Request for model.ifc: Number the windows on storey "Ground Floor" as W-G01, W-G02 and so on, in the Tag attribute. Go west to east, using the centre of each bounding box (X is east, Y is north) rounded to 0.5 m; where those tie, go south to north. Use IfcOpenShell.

First a look at what the model holds.

```python
import ifcopenshell
import ifcopenshell.util.element
import ifcopenshell.util.placement

model = ifcopenshell.open("model.ifc")
print(model.schema)
storey = next(s for s in model.by_type("IfcBuildingStorey") if s.Name == "Ground Floor")
windows = [e for e in ifcopenshell.util.element.get_decomposition(storey) if e.is_a("IfcWindow")]
for e in sorted(windows, key=lambda e: e.id()):
    origin = ifcopenshell.util.placement.get_local_placement(e.ObjectPlacement)[:3, 3]
    print(e.id(), e.Tag, e.Name, origin.round(2) + 0.0, sep=" | ")
```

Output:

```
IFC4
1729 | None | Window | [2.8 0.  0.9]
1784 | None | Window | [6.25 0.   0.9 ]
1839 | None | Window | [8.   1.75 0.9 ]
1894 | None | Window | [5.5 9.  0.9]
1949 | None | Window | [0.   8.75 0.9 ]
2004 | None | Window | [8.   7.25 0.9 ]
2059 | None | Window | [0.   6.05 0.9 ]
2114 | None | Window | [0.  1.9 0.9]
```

```python
import ifcopenshell
import ifcopenshell.geom
import ifcopenshell.util.element
import ifcopenshell.util.shape

model = ifcopenshell.open("model.ifc")
settings = ifcopenshell.geom.settings()
settings.set("use-world-coords", True)


def centre(element):
    shape = ifcopenshell.geom.create_shape(settings, element)
    return ifcopenshell.util.shape.get_bbox_centroid(shape.geometry)


storey = next(s for s in model.by_type("IfcBuildingStorey") if s.Name == "Ground Floor")
windows = [e for e in ifcopenshell.util.element.get_decomposition(storey) if e.is_a("IfcWindow")]

# Insertion points can sit at a corner or the storey origin, so sort by the geometry (in metres).
centres = {e: centre(e) for e in windows}
windows.sort(key=lambda e: (round(centres[e][0] / 0.5), centres[e][1]))

for i, e in enumerate(windows, start=1):
    number = f"W-G{i:02d}"
    e.Tag = number
    print(e.id(), number)

model.write("model_edited.ifc")
```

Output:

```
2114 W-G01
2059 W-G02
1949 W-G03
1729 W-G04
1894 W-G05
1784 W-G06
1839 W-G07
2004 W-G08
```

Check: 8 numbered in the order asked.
